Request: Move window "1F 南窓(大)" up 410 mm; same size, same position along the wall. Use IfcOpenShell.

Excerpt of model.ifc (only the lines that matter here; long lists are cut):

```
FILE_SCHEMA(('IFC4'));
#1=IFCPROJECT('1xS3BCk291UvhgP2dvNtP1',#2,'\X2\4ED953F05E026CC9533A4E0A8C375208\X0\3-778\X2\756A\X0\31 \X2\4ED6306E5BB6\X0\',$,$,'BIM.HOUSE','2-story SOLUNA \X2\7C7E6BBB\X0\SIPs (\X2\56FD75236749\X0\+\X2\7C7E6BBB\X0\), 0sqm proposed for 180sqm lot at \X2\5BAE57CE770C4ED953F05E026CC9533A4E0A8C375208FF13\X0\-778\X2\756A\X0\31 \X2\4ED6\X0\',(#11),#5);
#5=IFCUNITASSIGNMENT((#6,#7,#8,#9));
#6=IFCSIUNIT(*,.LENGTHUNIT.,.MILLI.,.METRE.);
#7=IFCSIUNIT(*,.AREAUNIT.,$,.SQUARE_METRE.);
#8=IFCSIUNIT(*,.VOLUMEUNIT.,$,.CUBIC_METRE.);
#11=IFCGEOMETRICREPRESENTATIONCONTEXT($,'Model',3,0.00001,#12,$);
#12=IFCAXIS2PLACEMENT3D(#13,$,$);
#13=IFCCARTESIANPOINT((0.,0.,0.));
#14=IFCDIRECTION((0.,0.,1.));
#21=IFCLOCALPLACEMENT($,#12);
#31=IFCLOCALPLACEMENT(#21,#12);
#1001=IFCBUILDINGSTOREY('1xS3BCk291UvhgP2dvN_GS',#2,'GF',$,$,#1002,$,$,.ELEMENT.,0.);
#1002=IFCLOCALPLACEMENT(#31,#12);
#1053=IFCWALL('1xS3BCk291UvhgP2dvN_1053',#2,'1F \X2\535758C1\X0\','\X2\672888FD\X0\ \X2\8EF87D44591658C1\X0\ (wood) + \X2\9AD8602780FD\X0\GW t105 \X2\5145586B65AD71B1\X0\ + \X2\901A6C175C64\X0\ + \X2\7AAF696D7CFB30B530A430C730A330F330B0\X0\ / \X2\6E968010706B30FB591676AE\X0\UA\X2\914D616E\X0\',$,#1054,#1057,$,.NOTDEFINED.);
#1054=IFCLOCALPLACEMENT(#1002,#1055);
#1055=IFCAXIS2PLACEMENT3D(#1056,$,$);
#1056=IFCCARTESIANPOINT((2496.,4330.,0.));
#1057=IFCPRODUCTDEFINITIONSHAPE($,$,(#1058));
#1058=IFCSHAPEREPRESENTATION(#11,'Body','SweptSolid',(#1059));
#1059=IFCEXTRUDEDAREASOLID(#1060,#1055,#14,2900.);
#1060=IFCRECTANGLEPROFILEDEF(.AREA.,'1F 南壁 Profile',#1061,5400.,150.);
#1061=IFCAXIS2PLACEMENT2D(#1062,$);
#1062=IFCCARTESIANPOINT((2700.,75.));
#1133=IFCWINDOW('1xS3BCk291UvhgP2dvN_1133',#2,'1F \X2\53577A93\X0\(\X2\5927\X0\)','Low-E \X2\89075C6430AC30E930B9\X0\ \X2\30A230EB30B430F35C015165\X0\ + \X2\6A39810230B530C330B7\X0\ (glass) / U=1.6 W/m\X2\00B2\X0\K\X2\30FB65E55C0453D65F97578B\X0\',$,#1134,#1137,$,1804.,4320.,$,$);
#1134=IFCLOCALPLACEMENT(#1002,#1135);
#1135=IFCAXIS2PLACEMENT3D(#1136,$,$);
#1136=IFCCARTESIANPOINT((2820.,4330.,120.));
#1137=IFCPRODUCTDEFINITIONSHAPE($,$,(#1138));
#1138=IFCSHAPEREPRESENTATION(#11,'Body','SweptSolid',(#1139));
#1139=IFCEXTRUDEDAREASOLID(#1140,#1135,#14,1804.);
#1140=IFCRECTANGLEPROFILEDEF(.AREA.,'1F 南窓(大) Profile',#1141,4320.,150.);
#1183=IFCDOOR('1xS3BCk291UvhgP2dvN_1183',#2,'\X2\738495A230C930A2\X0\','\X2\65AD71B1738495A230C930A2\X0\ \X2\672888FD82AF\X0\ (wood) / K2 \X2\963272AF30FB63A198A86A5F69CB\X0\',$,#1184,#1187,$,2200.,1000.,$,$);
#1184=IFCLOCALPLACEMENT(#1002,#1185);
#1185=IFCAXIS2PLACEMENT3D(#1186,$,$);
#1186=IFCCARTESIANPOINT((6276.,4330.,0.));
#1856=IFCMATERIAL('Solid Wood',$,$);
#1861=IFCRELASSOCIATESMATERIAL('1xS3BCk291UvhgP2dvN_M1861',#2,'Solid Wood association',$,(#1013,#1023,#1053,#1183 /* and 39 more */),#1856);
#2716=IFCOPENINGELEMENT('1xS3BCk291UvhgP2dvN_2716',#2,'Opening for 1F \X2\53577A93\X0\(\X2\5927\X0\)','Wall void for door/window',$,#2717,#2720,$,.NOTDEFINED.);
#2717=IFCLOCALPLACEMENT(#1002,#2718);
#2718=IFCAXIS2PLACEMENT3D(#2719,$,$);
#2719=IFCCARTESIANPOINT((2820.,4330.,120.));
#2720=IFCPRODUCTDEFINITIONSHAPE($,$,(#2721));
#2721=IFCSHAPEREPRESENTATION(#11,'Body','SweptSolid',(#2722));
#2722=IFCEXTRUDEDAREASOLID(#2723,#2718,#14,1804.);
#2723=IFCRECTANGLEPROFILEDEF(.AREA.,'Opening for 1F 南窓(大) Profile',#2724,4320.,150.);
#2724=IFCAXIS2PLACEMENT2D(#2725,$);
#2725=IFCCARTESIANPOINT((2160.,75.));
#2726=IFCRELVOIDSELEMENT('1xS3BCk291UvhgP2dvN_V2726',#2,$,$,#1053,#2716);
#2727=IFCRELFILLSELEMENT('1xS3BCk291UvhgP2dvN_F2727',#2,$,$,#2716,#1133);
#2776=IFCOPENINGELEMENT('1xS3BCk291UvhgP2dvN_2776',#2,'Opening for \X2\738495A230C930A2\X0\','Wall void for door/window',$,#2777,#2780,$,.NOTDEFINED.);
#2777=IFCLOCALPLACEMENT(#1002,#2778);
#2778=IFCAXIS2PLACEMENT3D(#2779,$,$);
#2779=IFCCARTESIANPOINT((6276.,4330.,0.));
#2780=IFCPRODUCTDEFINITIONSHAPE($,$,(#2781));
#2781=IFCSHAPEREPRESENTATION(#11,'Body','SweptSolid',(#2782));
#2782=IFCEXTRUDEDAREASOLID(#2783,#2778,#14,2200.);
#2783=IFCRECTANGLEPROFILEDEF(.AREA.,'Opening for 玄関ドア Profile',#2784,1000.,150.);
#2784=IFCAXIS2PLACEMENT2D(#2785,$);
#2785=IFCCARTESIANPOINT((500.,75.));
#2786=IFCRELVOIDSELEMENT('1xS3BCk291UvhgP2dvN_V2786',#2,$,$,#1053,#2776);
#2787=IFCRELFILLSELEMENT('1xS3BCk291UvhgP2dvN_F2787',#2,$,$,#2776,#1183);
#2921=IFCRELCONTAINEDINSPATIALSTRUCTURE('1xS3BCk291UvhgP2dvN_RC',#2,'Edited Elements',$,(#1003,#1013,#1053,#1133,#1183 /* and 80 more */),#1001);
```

```python
import numpy as np
import ifcopenshell
import ifcopenshell.api.geometry
import ifcopenshell.util.placement
import ifcopenshell.util.unit

model = ifcopenshell.open("model.ifc")
unit_scale = ifcopenshell.util.unit.calculate_unit_scale(model)

window = model.by_guid("1xS3BCk291UvhgP2dvN_1133")
opening = window.FillsVoids[0].RelatingOpeningElement
dz = 0.41 / unit_scale

shift = np.array([0.0, 0.0, dz])
# The window is not placed relative to its opening, so move both.
for product in (opening, window):
    matrix = ifcopenshell.util.placement.get_local_placement(product.ObjectPlacement)
    matrix[:3, 3] += shift
    ifcopenshell.api.geometry.edit_object_placement(model, product=product, matrix=matrix, is_si=False)

print(f"moved by {dz * unit_scale:+.3f} m")

model.write("model-out.ifc")
```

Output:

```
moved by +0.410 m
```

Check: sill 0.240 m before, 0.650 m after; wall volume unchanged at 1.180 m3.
